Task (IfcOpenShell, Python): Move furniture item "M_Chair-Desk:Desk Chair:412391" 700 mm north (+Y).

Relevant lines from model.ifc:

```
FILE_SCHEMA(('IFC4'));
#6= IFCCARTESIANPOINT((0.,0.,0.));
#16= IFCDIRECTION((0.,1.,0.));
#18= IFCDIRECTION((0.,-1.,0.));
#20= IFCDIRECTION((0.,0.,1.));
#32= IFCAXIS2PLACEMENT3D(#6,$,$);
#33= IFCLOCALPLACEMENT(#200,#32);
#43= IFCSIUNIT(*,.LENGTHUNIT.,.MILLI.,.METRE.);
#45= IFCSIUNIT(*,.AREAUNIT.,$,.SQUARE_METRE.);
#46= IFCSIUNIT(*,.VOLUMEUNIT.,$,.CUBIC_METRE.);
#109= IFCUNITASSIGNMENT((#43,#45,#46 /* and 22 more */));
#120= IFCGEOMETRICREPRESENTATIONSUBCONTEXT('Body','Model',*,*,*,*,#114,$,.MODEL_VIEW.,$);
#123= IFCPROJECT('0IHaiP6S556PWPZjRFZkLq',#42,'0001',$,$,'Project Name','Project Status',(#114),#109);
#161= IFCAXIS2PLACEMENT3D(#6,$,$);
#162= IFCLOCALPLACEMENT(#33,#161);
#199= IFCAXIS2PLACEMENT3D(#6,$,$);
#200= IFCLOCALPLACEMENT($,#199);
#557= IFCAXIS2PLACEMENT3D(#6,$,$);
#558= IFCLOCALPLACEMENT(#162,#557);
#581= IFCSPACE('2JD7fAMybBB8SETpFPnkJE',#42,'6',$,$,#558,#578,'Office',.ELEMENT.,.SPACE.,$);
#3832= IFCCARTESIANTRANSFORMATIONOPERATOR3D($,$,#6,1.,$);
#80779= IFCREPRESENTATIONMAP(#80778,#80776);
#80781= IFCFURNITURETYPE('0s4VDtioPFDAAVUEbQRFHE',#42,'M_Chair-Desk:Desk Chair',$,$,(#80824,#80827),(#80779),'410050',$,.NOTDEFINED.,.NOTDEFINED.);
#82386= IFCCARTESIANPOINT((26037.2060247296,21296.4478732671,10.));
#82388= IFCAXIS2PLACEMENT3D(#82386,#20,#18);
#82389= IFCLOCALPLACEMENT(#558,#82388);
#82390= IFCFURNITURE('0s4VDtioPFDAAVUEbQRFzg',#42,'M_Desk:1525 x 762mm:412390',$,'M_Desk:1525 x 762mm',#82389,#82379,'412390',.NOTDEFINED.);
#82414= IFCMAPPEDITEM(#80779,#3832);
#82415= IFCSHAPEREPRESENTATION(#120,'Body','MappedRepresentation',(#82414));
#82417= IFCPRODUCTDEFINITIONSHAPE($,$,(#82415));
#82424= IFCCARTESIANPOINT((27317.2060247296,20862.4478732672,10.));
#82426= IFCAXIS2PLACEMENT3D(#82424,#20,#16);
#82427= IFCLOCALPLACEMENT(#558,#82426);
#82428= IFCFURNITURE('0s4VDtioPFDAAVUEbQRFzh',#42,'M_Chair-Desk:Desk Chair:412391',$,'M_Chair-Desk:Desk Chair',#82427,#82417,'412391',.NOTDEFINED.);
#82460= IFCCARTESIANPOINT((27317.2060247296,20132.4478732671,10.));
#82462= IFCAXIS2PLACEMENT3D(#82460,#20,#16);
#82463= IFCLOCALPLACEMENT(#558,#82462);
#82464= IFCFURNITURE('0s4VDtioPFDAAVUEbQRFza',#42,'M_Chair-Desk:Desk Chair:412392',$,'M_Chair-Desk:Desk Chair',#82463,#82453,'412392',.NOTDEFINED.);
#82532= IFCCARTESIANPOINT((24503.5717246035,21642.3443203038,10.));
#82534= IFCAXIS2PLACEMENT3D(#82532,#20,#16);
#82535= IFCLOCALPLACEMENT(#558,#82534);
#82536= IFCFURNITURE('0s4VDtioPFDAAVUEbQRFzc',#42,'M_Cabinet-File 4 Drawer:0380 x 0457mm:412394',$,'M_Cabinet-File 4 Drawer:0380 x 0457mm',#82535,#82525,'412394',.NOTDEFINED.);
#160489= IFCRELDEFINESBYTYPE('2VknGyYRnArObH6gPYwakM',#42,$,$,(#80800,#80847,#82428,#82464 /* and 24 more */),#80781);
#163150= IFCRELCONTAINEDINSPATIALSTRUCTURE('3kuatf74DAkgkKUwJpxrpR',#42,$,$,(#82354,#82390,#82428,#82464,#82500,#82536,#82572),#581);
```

```python
import ifcopenshell
import ifcopenshell.api.geometry
import ifcopenshell.util.placement

model = ifcopenshell.open("model.ifc")

item = model.by_id(82428)
matrix = ifcopenshell.util.placement.get_local_placement(item.ObjectPlacement)
matrix[1, 3] += 700.0
ifcopenshell.api.geometry.edit_object_placement(model, product=item, matrix=matrix, is_si=False)

print(ifcopenshell.util.placement.get_local_placement(item.ObjectPlacement).round(3) + 0.0)

model.write("model-out.ifc")
```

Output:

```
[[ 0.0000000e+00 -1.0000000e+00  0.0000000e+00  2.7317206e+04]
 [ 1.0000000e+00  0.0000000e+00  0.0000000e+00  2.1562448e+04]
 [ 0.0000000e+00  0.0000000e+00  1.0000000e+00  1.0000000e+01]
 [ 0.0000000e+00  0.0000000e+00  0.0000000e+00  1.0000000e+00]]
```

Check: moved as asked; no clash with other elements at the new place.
